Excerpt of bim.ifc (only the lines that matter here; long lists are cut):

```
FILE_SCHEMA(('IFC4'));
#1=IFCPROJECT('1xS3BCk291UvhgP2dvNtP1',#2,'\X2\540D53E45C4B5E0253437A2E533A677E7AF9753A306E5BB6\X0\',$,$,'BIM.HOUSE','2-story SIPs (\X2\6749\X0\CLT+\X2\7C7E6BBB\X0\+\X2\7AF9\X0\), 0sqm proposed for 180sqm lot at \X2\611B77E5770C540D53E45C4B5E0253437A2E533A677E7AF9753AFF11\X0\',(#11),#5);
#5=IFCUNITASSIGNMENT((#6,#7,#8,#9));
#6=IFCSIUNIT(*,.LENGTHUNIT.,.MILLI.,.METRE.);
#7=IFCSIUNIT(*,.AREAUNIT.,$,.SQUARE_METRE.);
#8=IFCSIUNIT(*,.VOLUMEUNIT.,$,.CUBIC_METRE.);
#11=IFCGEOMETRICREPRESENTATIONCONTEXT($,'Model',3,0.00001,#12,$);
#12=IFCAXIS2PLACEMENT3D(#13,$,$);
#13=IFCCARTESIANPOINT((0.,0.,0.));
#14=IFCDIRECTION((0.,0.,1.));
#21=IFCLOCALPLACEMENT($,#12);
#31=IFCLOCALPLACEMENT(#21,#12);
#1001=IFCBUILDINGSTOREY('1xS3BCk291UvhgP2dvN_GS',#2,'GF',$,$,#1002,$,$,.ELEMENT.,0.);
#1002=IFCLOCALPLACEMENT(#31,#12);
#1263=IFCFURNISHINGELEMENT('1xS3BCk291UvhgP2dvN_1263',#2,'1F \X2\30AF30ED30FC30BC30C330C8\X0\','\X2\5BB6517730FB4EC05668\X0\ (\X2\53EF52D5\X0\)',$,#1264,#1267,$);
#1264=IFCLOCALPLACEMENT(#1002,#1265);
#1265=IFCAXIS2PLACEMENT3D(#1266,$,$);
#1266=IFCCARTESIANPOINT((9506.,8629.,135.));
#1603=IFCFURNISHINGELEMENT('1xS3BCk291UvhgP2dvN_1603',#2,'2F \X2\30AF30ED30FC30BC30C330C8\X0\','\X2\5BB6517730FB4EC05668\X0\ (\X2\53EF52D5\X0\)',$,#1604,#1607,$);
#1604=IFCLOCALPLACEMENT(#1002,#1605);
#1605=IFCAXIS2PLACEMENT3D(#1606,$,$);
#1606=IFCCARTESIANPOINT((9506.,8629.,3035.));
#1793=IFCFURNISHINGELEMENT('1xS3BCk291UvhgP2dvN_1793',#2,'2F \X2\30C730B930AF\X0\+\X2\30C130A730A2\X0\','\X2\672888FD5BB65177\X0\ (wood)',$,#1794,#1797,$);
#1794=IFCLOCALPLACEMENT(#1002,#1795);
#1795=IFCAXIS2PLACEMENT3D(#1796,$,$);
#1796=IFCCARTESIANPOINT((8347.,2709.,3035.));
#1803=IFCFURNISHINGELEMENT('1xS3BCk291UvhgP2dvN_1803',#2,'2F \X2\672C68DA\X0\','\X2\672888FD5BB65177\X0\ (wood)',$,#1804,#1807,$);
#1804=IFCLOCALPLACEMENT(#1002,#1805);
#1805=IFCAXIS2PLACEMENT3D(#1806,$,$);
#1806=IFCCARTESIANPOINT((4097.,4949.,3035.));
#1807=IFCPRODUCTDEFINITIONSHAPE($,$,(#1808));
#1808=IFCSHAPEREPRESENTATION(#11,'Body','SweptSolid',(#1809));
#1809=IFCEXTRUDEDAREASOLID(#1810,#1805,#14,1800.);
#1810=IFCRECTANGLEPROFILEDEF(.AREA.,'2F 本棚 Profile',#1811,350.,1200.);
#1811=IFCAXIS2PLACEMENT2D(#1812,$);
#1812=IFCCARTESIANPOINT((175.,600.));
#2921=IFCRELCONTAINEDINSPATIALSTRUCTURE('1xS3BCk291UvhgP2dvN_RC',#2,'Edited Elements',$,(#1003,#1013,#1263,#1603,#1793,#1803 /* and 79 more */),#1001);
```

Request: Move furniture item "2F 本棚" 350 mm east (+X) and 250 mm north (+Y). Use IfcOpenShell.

```python
import ifcopenshell
import ifcopenshell.api.geometry
import ifcopenshell.util.placement

model = ifcopenshell.open("bim.ifc")

item = model.by_id(1803)
matrix = ifcopenshell.util.placement.get_local_placement(item.ObjectPlacement)
matrix[0, 3] += 350.0
matrix[1, 3] += 250.0
ifcopenshell.api.geometry.edit_object_placement(model, product=item, matrix=matrix, is_si=False)

print(ifcopenshell.util.placement.get_local_placement(item.ObjectPlacement).round(3) + 0.0)

model.write("bim-out.ifc")
```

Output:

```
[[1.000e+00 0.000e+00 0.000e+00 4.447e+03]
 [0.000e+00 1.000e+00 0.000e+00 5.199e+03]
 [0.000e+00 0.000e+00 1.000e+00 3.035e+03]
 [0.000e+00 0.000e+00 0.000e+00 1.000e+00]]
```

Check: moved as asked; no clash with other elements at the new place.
